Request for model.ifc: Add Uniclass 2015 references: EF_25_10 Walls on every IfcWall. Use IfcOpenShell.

First a look at what the model holds.

```python
import ifcopenshell

model = ifcopenshell.open("model.ifc")
print(model.schema)
print("classifications:", [c.Name for c in model.by_type("IfcClassification")])
for ifc_class in ("IfcDoor", "IfcRoof", "IfcStair", "IfcWall", "IfcWindow"):
    print(ifc_class, len(model.by_type(ifc_class)))
```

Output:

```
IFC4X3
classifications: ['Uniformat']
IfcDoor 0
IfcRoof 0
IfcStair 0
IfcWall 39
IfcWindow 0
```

```python
import ifcopenshell
import ifcopenshell.api.classification

model = ifcopenshell.open("model.ifc")

system = ifcopenshell.api.classification.add_classification(model, classification="Uniclass 2015")

codes = {
    "IfcWall": ("EF_25_10", "Walls"),
}
for ifc_class, (code, name) in codes.items():
    products = model.by_type(ifc_class)
    ifcopenshell.api.classification.add_reference(
        model, products=products, classification=system, identification=code, name=name
    )
    print(code, len(products))

model.write("model_rev.ifc")
```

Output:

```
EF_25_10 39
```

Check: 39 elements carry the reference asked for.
